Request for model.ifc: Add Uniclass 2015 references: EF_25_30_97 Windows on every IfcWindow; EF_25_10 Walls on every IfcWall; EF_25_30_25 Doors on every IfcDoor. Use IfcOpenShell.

First a look at what the model holds.

```python
import ifcopenshell

model = ifcopenshell.open("model.ifc")
print(model.schema)
print("classifications:", [c.Name for c in model.by_type("IfcClassification")])
for ifc_class in ("IfcDoor", "IfcRoof", "IfcStair", "IfcWall", "IfcWindow"):
    print(ifc_class, len(model.by_type(ifc_class)))
```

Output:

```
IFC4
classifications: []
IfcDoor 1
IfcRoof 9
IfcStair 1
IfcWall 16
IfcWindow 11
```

```python
import ifcopenshell
import ifcopenshell.api.classification

model = ifcopenshell.open("model.ifc")

system = ifcopenshell.api.classification.add_classification(model, classification="Uniclass 2015")

codes = {
    "IfcWindow": ("EF_25_30_97", "Windows"),
    "IfcWall": ("EF_25_10", "Walls"),
    "IfcDoor": ("EF_25_30_25", "Doors"),
}
for ifc_class, (code, name) in codes.items():
    products = model.by_type(ifc_class)
    ifcopenshell.api.classification.add_reference(
        model, products=products, classification=system, identification=code, name=name
    )
    print(code, len(products))

model.write("model_edited.ifc")
```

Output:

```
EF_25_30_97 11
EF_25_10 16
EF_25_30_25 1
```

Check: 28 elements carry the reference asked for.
